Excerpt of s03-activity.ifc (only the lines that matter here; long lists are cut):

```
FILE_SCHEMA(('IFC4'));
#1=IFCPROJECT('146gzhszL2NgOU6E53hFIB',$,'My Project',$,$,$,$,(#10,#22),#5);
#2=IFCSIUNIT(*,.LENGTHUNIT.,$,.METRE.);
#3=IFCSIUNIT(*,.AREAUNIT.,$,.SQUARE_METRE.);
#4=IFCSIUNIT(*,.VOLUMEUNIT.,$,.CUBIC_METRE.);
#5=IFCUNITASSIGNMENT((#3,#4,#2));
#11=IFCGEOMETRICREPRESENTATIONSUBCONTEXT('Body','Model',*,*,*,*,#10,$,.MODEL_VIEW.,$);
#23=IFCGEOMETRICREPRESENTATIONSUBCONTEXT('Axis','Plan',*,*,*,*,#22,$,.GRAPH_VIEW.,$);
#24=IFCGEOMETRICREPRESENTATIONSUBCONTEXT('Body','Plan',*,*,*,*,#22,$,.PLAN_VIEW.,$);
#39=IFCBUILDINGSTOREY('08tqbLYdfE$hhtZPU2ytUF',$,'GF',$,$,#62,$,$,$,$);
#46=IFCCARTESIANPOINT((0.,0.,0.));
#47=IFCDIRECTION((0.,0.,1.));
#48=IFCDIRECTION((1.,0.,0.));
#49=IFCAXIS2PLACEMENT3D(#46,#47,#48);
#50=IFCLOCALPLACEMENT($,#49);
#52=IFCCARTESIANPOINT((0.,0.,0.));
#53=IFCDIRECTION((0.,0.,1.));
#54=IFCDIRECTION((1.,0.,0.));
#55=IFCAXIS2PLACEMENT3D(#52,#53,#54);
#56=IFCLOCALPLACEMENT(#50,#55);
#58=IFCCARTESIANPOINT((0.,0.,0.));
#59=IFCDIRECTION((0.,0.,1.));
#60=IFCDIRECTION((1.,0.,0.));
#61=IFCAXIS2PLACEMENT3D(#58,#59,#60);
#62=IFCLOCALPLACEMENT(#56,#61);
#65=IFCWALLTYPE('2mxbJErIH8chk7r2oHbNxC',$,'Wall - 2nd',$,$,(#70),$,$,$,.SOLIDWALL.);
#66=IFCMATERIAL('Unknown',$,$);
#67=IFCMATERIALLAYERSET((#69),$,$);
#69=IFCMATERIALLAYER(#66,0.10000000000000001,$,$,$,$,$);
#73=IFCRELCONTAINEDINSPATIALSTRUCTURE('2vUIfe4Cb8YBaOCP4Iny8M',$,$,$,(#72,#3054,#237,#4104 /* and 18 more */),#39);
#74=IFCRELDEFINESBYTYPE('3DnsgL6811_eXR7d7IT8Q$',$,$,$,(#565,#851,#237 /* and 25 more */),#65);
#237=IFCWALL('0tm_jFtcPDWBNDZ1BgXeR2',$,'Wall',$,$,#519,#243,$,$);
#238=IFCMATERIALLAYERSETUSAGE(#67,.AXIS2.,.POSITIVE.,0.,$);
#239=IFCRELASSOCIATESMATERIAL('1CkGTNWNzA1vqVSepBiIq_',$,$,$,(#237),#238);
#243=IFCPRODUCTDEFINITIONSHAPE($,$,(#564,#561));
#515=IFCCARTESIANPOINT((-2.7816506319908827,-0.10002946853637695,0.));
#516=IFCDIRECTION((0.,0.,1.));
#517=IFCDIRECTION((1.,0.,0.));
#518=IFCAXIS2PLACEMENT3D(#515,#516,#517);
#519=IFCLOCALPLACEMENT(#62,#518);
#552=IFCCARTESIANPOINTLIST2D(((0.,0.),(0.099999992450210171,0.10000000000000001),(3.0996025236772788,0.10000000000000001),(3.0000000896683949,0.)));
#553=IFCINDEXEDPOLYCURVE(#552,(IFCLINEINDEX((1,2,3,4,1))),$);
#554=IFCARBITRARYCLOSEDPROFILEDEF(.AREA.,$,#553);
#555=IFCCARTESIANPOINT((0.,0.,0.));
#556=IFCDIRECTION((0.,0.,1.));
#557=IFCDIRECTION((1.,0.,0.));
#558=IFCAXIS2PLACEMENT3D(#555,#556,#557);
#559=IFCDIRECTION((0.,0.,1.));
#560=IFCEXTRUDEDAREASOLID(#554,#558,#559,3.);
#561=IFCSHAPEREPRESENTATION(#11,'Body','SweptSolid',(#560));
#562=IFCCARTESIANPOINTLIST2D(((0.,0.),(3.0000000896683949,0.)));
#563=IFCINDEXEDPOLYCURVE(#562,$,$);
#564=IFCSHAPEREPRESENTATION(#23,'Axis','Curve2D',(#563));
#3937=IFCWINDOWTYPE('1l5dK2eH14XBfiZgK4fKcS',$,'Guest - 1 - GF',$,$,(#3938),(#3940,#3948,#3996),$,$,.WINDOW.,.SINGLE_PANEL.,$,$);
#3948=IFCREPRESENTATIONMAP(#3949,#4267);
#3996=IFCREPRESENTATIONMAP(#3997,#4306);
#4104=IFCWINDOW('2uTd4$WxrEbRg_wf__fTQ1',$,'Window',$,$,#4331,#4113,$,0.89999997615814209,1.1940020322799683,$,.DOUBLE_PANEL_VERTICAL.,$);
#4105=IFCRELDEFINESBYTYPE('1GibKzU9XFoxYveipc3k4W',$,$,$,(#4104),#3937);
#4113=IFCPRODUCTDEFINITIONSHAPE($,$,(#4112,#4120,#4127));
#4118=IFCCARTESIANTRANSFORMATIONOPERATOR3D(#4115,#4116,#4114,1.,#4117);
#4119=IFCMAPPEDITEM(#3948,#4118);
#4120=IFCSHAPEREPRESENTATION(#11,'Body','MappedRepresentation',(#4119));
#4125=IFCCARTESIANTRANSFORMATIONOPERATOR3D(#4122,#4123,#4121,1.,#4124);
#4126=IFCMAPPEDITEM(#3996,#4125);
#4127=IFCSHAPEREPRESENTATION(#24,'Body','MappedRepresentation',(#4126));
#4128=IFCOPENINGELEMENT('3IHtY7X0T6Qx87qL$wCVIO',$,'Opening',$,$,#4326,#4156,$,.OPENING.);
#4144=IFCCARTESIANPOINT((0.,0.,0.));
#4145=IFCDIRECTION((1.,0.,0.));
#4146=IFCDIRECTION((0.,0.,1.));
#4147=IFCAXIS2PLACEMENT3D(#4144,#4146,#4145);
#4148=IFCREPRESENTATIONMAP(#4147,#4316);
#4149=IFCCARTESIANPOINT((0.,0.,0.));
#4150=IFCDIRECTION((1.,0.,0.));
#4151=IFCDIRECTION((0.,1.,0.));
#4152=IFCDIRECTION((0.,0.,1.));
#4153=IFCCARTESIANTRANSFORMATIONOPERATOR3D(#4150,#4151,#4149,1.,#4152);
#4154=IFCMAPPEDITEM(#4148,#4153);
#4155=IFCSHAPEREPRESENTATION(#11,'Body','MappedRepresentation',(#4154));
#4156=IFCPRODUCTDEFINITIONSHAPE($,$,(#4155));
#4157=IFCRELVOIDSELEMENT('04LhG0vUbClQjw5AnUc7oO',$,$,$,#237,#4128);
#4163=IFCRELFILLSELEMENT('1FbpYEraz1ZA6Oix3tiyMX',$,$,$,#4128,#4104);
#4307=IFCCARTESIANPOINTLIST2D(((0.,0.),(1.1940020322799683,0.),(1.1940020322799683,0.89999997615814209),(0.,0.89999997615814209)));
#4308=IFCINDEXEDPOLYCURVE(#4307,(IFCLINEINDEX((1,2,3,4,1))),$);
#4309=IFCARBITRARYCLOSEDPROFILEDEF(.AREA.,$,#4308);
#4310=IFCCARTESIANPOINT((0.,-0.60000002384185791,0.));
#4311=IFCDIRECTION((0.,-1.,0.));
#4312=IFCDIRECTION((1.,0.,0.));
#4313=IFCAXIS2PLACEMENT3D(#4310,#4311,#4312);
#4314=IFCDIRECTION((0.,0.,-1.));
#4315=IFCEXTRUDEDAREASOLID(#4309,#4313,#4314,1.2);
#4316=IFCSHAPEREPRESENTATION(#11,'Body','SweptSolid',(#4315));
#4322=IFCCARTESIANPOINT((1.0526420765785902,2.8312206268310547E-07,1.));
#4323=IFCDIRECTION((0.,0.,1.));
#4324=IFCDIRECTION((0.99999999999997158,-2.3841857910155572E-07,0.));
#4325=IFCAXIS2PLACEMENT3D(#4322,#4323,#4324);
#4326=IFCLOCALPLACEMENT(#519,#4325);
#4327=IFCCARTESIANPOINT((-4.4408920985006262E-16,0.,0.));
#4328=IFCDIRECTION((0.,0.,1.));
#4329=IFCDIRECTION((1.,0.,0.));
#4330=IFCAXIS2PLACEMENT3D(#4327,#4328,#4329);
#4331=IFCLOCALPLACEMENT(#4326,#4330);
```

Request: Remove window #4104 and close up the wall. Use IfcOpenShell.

```python
import ifcopenshell
import ifcopenshell.api.feature
import ifcopenshell.api.root
import ifcopenshell.geom
import ifcopenshell.util.shape

model = ifcopenshell.open("s03-activity.ifc")
settings = ifcopenshell.geom.settings()


def volume(element):
    """Net volume in cubic metres, openings subtracted."""
    shape = ifcopenshell.geom.create_shape(settings, element)
    return ifcopenshell.util.shape.get_volume(shape.geometry)


window = model.by_guid("2uTd4$WxrEbRg_wf__fTQ1")
opening = window.FillsVoids[0].RelatingOpeningElement
wall = opening.VoidsElements[0].RelatingBuildingElement
before = volume(wall)

ifcopenshell.api.root.remove_product(model, product=window)
ifcopenshell.api.feature.remove_feature(model, feature=opening)

after = volume(wall)

print(f"wall volume {before:.3f} -> {after:.3f} m3")

model.write("s03-activity-out.ifc")
```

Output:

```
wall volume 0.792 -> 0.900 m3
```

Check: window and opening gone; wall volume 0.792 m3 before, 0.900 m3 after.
